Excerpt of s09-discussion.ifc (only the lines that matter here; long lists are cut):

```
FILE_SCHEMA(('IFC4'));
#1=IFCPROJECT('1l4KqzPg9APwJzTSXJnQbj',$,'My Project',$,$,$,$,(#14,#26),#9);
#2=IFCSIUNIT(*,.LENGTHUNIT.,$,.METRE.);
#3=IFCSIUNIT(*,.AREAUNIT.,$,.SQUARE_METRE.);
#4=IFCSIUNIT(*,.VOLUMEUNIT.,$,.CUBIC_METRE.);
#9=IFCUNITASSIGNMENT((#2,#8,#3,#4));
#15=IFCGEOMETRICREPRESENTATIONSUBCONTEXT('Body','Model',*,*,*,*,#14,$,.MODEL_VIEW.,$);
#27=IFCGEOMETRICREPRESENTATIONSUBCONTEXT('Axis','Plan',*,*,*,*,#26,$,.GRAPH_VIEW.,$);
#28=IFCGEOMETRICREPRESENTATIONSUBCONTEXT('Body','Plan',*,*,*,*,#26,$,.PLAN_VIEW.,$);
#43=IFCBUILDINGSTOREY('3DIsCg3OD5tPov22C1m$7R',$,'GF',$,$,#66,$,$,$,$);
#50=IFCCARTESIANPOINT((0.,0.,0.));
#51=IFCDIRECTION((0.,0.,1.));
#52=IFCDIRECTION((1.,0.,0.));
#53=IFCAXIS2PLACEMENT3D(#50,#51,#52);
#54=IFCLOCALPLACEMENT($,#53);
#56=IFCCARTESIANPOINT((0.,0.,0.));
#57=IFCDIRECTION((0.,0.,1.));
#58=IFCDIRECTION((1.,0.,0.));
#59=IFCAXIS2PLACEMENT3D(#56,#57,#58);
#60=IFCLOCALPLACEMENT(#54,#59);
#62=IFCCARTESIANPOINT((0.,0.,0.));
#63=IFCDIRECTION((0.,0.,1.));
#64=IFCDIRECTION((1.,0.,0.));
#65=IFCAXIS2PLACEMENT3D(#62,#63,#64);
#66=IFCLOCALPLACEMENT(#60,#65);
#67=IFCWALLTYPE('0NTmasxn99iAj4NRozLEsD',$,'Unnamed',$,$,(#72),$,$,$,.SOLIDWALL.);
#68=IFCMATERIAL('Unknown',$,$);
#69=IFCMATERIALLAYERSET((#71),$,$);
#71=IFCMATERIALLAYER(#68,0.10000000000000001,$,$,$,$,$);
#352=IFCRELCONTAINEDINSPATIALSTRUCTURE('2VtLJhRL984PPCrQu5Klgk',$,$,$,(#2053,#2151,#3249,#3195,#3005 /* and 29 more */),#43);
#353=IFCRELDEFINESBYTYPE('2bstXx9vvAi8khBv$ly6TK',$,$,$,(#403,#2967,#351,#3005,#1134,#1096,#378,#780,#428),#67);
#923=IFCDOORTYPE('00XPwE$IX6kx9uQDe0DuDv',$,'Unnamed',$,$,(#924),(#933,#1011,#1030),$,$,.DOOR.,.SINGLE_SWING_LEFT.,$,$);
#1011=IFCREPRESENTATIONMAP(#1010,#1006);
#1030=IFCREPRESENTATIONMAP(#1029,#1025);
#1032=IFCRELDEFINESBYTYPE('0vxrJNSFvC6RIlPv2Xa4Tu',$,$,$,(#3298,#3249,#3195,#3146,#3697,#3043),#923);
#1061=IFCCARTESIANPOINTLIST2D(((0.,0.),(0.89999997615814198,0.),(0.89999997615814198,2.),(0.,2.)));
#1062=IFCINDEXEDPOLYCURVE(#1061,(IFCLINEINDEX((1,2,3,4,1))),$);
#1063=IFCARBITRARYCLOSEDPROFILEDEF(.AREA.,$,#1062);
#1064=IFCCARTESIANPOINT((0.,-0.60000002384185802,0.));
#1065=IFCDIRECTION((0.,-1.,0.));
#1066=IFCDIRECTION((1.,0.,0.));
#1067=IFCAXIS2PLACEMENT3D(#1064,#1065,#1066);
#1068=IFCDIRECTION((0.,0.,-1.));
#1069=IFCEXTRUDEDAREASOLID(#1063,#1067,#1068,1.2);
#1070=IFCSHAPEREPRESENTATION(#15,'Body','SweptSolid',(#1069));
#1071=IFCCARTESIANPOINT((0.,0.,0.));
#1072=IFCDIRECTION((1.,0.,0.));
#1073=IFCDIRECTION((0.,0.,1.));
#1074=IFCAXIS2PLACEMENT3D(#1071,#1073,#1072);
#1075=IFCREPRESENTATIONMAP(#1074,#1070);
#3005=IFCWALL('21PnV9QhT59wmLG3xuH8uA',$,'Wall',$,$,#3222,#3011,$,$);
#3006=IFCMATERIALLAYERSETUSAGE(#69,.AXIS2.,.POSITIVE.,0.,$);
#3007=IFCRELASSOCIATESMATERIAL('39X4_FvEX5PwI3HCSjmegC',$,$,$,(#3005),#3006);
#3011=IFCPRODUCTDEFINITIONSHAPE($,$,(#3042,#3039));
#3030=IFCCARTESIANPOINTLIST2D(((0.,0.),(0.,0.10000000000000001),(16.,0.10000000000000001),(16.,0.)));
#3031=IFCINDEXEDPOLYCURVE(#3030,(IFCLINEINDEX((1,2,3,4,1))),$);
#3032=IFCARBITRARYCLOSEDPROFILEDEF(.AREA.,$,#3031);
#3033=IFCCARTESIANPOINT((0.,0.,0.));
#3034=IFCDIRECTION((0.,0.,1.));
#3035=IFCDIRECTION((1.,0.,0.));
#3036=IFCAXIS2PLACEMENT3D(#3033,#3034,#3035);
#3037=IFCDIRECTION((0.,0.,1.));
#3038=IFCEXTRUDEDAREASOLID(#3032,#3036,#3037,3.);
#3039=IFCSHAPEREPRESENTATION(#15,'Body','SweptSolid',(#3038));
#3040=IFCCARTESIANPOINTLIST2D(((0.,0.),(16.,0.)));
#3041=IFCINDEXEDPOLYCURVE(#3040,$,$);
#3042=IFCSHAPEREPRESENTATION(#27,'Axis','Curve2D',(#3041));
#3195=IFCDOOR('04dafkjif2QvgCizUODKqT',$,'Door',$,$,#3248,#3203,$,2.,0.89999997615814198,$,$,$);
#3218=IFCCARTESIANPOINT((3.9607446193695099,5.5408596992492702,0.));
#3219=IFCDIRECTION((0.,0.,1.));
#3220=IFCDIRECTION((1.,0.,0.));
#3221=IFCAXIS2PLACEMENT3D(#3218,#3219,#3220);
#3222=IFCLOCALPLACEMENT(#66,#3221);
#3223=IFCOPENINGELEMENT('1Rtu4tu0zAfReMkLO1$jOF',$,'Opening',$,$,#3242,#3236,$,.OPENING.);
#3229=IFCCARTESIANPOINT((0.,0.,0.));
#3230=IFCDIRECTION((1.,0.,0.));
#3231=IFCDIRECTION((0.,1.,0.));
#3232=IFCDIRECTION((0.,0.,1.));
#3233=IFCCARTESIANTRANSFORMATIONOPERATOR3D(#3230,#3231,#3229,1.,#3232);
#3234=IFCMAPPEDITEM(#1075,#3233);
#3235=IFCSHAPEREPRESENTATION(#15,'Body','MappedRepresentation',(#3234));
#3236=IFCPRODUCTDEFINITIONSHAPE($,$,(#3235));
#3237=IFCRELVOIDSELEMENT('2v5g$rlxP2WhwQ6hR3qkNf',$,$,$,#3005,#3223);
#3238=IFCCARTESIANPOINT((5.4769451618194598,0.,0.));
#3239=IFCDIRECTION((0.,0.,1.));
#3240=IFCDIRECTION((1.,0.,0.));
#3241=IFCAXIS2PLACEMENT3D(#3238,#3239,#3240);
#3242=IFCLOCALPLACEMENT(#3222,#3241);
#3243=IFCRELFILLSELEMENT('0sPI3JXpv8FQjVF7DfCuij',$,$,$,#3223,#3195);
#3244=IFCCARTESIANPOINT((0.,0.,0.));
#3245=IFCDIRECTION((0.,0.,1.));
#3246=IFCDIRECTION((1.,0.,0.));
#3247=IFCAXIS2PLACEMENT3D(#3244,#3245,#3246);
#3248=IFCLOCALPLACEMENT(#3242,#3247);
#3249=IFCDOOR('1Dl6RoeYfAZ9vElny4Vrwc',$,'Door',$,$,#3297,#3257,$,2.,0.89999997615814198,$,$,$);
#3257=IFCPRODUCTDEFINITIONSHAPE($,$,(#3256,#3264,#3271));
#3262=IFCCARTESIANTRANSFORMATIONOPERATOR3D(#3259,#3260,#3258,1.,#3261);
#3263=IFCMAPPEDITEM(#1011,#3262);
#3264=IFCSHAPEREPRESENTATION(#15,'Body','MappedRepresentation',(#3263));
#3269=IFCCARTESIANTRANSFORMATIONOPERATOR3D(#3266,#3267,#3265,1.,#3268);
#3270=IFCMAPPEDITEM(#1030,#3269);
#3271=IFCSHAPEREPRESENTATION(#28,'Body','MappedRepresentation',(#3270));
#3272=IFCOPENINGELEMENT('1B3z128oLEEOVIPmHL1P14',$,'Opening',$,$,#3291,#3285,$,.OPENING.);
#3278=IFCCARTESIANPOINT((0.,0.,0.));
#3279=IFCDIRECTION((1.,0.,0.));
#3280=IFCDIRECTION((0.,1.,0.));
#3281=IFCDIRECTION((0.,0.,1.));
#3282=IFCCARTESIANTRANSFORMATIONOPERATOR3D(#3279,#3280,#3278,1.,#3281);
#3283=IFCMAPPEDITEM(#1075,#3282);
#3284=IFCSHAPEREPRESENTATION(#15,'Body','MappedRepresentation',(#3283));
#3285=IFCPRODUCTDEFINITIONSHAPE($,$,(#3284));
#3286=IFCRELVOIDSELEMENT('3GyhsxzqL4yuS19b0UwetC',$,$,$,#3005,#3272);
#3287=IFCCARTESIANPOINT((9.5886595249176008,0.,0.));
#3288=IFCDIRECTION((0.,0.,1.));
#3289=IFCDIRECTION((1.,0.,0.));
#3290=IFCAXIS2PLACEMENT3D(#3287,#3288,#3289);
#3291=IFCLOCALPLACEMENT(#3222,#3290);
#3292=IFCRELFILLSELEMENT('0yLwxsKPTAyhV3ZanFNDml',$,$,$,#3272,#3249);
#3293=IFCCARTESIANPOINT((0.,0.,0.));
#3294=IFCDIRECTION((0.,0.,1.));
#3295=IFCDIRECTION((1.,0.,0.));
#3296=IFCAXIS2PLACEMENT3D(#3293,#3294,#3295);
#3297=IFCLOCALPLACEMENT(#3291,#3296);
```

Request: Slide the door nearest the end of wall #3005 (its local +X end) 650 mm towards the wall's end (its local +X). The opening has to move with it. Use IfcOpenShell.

```python
import ifcopenshell
import ifcopenshell.api.geometry
import ifcopenshell.util.placement
import ifcopenshell.util.unit

model = ifcopenshell.open("s09-discussion.ifc")
unit_scale = ifcopenshell.util.unit.calculate_unit_scale(model)

door = model.by_guid("1Dl6RoeYfAZ9vElny4Vrwc")
opening = door.FillsVoids[0].RelatingOpeningElement
wall = opening.VoidsElements[0].RelatingBuildingElement

wall_matrix = ifcopenshell.util.placement.get_local_placement(wall.ObjectPlacement)
shift = wall_matrix[:3, 0] * 0.65 / unit_scale
before = ifcopenshell.util.placement.get_local_placement(door.ObjectPlacement)[:3, 3].copy()

# The door is placed relative to its opening, so it follows when the opening moves.
matrix = ifcopenshell.util.placement.get_local_placement(opening.ObjectPlacement)
matrix[:3, 3] += shift
ifcopenshell.api.geometry.edit_object_placement(
    model, product=opening, matrix=matrix, is_si=False, should_transform_children=True
)

after = ifcopenshell.util.placement.get_local_placement(door.ObjectPlacement)[:3, 3]
print("door moved by", (after - before).round(3) + 0.0)

model.write("s09-discussion_updated.ifc")
```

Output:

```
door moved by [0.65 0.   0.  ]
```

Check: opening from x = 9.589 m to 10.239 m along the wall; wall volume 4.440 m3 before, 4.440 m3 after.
